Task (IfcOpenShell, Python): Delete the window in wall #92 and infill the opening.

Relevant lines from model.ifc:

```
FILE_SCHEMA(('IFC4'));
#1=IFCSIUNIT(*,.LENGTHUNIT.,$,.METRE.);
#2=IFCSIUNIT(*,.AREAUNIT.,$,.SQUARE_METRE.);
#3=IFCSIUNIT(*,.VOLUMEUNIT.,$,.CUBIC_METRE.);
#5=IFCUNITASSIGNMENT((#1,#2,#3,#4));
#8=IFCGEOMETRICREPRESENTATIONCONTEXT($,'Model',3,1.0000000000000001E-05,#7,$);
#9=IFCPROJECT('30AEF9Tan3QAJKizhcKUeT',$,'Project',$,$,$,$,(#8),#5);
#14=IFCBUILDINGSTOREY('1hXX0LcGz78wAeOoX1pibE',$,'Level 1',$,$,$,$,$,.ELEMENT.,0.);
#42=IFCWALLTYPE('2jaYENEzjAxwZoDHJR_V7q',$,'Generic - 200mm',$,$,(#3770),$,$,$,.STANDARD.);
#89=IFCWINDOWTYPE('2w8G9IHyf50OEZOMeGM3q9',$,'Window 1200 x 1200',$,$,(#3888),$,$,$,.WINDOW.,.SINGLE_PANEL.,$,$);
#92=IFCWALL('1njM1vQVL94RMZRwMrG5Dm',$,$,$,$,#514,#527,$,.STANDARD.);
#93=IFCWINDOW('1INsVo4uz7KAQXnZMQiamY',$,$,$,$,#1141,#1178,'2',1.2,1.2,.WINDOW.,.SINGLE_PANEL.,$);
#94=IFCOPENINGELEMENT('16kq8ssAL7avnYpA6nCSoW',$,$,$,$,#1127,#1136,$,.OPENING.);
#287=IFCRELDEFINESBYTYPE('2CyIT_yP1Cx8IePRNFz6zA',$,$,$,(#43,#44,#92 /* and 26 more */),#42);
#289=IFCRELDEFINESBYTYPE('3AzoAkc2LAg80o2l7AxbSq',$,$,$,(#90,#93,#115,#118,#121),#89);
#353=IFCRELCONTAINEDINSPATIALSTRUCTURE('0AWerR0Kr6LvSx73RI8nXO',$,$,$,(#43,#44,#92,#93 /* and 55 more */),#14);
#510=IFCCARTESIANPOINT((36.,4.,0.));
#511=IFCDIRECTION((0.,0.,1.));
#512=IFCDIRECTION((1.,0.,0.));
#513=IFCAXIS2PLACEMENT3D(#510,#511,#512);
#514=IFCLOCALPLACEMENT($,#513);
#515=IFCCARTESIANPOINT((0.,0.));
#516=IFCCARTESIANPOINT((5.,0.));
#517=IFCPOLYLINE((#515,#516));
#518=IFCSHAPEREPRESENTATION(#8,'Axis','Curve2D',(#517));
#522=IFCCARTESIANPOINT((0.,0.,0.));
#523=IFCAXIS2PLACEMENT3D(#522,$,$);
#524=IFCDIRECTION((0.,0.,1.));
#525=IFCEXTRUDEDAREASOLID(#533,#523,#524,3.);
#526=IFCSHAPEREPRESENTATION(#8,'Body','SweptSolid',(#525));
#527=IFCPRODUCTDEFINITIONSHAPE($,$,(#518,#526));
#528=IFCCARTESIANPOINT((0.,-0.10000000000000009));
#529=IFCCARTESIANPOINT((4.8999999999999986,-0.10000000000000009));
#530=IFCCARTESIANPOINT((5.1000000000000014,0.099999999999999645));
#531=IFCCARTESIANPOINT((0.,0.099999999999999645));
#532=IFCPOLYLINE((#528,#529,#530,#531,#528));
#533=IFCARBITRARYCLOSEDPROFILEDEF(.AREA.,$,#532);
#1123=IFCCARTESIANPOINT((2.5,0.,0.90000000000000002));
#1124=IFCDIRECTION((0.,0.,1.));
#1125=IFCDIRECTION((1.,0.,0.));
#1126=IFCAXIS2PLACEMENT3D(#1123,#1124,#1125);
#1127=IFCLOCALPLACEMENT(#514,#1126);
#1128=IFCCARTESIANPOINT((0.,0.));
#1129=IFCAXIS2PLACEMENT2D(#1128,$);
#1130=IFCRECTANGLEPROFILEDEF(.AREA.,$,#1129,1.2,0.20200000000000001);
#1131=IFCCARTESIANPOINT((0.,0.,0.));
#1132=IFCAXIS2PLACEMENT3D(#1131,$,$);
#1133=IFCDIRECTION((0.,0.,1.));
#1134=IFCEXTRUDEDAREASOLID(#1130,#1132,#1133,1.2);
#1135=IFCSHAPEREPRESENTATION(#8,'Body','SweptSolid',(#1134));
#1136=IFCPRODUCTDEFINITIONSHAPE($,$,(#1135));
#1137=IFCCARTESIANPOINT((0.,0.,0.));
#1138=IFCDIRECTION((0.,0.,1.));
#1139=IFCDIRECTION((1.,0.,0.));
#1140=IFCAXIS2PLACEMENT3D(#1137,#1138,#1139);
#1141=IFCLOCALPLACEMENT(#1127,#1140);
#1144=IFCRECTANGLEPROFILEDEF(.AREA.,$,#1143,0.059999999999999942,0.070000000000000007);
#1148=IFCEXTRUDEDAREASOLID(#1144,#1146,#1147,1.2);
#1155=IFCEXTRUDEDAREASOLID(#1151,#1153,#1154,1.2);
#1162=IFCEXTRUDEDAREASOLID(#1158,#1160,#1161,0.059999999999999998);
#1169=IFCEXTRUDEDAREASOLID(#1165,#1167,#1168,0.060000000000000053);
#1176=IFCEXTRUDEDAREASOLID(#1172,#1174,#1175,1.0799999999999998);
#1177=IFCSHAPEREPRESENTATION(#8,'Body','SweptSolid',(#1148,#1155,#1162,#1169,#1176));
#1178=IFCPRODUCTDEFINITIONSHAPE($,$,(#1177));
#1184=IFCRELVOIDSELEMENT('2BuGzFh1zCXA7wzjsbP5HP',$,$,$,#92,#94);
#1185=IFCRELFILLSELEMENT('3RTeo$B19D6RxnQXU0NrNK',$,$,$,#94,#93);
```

```python
import ifcopenshell
import ifcopenshell.api.feature
import ifcopenshell.api.root
import ifcopenshell.geom
import ifcopenshell.util.shape

model = ifcopenshell.open("model.ifc")
settings = ifcopenshell.geom.settings()


def volume(element):
    """Net volume in cubic metres, openings subtracted."""
    shape = ifcopenshell.geom.create_shape(settings, element)
    return ifcopenshell.util.shape.get_volume(shape.geometry)


window = model.by_id(93)
opening = window.FillsVoids[0].RelatingOpeningElement
wall = opening.VoidsElements[0].RelatingBuildingElement
before = volume(wall)

ifcopenshell.api.root.remove_product(model, product=window)
ifcopenshell.api.feature.remove_feature(model, feature=opening)

after = volume(wall)

print(f"wall volume {before:.3f} -> {after:.3f} m3")

model.write("model_updated.ifc")
```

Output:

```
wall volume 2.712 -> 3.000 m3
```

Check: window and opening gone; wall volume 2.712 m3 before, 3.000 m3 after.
